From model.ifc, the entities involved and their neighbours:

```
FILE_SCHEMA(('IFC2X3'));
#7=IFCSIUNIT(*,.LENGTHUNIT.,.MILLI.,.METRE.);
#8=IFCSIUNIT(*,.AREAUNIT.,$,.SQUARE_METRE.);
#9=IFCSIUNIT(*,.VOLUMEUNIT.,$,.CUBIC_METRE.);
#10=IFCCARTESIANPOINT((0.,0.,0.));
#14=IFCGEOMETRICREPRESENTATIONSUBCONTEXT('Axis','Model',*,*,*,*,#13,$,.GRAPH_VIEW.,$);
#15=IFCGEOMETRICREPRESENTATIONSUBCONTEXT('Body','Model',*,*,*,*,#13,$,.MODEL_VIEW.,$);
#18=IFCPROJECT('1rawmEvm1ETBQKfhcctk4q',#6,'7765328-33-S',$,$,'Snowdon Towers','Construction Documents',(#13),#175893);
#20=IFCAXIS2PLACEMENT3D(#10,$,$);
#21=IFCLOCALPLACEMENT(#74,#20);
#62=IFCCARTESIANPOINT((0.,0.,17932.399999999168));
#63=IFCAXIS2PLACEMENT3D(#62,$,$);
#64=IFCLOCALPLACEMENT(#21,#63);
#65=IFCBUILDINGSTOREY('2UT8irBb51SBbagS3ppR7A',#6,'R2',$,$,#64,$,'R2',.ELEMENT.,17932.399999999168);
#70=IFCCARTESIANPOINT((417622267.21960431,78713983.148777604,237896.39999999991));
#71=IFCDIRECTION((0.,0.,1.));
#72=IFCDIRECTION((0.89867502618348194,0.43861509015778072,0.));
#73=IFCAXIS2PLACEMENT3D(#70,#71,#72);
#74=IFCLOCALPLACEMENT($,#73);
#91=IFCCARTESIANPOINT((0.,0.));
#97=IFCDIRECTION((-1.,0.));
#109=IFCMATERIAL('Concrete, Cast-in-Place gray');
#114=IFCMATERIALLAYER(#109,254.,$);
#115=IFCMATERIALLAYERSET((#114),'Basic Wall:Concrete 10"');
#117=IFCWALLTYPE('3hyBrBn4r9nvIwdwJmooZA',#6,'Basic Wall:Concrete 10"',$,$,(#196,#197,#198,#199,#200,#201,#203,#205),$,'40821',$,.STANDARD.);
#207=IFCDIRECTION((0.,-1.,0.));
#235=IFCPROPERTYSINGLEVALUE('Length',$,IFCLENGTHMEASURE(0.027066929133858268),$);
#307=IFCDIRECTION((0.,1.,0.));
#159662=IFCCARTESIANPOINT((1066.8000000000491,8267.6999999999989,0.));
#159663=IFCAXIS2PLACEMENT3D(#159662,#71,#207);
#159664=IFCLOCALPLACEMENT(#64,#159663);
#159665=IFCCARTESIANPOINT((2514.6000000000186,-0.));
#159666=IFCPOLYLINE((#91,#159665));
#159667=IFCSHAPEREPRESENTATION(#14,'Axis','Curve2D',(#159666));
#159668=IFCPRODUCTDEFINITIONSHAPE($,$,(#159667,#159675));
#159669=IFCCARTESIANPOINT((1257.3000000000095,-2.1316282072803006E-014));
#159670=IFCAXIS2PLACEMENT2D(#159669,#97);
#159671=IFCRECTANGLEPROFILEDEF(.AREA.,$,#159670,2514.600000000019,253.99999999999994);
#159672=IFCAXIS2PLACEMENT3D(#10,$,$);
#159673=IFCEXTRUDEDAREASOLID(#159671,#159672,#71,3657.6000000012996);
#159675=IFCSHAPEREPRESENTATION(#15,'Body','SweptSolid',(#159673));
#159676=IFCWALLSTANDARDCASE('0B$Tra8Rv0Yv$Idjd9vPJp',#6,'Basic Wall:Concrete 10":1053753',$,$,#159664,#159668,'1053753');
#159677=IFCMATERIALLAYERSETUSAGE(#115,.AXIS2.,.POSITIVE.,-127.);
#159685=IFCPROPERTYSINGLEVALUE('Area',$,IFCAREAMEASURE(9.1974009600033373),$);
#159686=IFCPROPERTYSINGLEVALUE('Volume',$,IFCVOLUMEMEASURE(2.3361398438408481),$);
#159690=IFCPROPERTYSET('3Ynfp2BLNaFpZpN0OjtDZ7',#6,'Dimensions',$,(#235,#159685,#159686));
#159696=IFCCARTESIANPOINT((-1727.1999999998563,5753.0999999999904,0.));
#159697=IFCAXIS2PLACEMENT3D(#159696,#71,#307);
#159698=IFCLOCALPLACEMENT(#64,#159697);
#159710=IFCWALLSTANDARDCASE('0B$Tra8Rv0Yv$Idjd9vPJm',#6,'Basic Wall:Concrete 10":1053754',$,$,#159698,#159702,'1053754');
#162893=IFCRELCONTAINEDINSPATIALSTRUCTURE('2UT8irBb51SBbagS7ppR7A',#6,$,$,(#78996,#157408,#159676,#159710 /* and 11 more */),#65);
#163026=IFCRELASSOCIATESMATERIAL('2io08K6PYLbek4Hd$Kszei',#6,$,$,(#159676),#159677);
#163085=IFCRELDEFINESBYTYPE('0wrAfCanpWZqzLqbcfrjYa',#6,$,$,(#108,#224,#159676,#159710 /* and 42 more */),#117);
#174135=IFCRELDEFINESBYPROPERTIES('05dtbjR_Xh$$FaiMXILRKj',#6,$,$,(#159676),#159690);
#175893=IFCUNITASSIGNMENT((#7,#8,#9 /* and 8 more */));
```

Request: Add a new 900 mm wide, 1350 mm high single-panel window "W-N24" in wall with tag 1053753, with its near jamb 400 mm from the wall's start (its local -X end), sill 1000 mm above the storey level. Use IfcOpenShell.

```python
import numpy as np
import ifcopenshell
import ifcopenshell.api.feature
import ifcopenshell.api.geometry
import ifcopenshell.api.pset
import ifcopenshell.api.root
import ifcopenshell.api.spatial
import ifcopenshell.api.type
import ifcopenshell.geom
import ifcopenshell.util.element
import ifcopenshell.util.placement
import ifcopenshell.util.representation
import ifcopenshell.util.shape
import ifcopenshell.util.unit

model = ifcopenshell.open("model.ifc")
unit_scale = ifcopenshell.util.unit.calculate_unit_scale(model)
area_scale = ifcopenshell.util.unit.calculate_unit_scale(model, "AREAUNIT")
volume_scale = ifcopenshell.util.unit.calculate_unit_scale(model, "VOLUMEUNIT")
settings = ifcopenshell.geom.settings()


def volume(element):
    """Net volume in cubic metres, openings subtracted."""
    shape = ifcopenshell.geom.create_shape(settings, element)
    return ifcopenshell.util.shape.get_volume(shape.geometry)


wall = model.by_guid("0B$Tra8Rv0Yv$Idjd9vPJp")
storey = ifcopenshell.util.element.get_container(wall, ifc_class="IfcBuildingStorey")
context = ifcopenshell.util.representation.get_context(model, "Model", "Body", "MODEL_VIEW")
before = volume(wall)

width, height, from_end, sill = 0.9, 1.35, 0.4, 1  # metres

# The wall runs along its own X axis, and the end named is its -X end.
wall_shape = ifcopenshell.geom.create_shape(settings, wall)
x, y, z = ifcopenshell.util.shape.get_vertices(wall_shape.geometry).T
start = x.min() + from_end
face, thickness = float(y.min()), float(y.max() - y.min())
wall_matrix = ifcopenshell.util.placement.get_local_placement(wall.ObjectPlacement)
level = ifcopenshell.util.placement.get_local_placement(storey.ObjectPlacement)[2, 3]


def in_wall(x, y):
    """Placement at x, y metres in the wall's axes, at sill height."""
    matrix = wall_matrix.copy()
    matrix[:, 3] = wall_matrix @ np.array([x / unit_scale, y / unit_scale, 0.0, 1.0])
    matrix[2, 3] = level + sill / unit_scale
    return matrix


# Opening: a box that overshoots both wall faces by 50 mm.
opening = ifcopenshell.api.root.create_entity(model, ifc_class="IfcOpeningElement")
box = ifcopenshell.api.geometry.add_wall_representation(
    model, context=context, length=width, height=height, thickness=thickness + 0.1
)
ifcopenshell.api.geometry.assign_representation(model, product=opening, representation=box)
ifcopenshell.api.geometry.edit_object_placement(model, product=opening, matrix=in_wall(start, face - 0.05), is_si=False)
ifcopenshell.api.feature.add_feature(model, feature=opening, element=wall)

window = ifcopenshell.api.root.create_entity(model, ifc_class="IfcWindow", name="W-N24")
window.OverallWidth, window.OverallHeight = width / unit_scale, height / unit_scale
body = ifcopenshell.api.geometry.add_window_representation(
    model,
    context=context,
    overall_width=window.OverallWidth,
    overall_height=window.OverallHeight,
    partition_type="SINGLE_PANEL",
)
ifcopenshell.api.geometry.assign_representation(model, product=window, representation=body)
ifcopenshell.api.spatial.assign_container(model, products=[window], relating_structure=storey)
fills = ifcopenshell.api.feature.add_filling(model, opening=opening, element=window)
fills.OwnerHistory = window.OwnerHistory  # required in IFC2X3

# IFC2X3 keeps the operation on the window style.
style = ifcopenshell.api.root.create_entity(model, ifc_class="IfcWindowStyle", name="W-N24")
style.OperationType, style.ConstructionType = "SINGLE_PANEL", "NOTDEFINED"
style.ParameterTakesPrecedence = style.Sizeable = False
ifcopenshell.api.type.assign_type(model, related_objects=[window], relating_type=style)

# Centre the window in the wall's thickness.
ifcopenshell.api.geometry.edit_object_placement(model, product=window, matrix=in_wall(start, face), is_si=False)
window_shape = ifcopenshell.geom.create_shape(settings, window)
depth = ifcopenshell.util.shape.get_vertices(window_shape.geometry)[:, 1]
offset = face + thickness / 2 - (depth.min() + depth.max()) / 2
ifcopenshell.api.geometry.edit_object_placement(model, product=window, matrix=in_wall(start, offset), is_si=False)

after = volume(wall)

# Update the wall's stored quantities.
pset = model.by_id(ifcopenshell.util.element.get_pset(wall, "Dimensions", should_inherit=False)["id"])
ifcopenshell.api.pset.edit_pset(model, pset=pset, properties={
    "Area": model.create_entity("IfcAreaMeasure", after / thickness / area_scale),
    "Volume": model.create_entity("IfcVolumeMeasure", after / volume_scale),
})

print(f"wall volume {before:.3f} -> {after:.3f} m3")

model.write("model_v2.ifc")
```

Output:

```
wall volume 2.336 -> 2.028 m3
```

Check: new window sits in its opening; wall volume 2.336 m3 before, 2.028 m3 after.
